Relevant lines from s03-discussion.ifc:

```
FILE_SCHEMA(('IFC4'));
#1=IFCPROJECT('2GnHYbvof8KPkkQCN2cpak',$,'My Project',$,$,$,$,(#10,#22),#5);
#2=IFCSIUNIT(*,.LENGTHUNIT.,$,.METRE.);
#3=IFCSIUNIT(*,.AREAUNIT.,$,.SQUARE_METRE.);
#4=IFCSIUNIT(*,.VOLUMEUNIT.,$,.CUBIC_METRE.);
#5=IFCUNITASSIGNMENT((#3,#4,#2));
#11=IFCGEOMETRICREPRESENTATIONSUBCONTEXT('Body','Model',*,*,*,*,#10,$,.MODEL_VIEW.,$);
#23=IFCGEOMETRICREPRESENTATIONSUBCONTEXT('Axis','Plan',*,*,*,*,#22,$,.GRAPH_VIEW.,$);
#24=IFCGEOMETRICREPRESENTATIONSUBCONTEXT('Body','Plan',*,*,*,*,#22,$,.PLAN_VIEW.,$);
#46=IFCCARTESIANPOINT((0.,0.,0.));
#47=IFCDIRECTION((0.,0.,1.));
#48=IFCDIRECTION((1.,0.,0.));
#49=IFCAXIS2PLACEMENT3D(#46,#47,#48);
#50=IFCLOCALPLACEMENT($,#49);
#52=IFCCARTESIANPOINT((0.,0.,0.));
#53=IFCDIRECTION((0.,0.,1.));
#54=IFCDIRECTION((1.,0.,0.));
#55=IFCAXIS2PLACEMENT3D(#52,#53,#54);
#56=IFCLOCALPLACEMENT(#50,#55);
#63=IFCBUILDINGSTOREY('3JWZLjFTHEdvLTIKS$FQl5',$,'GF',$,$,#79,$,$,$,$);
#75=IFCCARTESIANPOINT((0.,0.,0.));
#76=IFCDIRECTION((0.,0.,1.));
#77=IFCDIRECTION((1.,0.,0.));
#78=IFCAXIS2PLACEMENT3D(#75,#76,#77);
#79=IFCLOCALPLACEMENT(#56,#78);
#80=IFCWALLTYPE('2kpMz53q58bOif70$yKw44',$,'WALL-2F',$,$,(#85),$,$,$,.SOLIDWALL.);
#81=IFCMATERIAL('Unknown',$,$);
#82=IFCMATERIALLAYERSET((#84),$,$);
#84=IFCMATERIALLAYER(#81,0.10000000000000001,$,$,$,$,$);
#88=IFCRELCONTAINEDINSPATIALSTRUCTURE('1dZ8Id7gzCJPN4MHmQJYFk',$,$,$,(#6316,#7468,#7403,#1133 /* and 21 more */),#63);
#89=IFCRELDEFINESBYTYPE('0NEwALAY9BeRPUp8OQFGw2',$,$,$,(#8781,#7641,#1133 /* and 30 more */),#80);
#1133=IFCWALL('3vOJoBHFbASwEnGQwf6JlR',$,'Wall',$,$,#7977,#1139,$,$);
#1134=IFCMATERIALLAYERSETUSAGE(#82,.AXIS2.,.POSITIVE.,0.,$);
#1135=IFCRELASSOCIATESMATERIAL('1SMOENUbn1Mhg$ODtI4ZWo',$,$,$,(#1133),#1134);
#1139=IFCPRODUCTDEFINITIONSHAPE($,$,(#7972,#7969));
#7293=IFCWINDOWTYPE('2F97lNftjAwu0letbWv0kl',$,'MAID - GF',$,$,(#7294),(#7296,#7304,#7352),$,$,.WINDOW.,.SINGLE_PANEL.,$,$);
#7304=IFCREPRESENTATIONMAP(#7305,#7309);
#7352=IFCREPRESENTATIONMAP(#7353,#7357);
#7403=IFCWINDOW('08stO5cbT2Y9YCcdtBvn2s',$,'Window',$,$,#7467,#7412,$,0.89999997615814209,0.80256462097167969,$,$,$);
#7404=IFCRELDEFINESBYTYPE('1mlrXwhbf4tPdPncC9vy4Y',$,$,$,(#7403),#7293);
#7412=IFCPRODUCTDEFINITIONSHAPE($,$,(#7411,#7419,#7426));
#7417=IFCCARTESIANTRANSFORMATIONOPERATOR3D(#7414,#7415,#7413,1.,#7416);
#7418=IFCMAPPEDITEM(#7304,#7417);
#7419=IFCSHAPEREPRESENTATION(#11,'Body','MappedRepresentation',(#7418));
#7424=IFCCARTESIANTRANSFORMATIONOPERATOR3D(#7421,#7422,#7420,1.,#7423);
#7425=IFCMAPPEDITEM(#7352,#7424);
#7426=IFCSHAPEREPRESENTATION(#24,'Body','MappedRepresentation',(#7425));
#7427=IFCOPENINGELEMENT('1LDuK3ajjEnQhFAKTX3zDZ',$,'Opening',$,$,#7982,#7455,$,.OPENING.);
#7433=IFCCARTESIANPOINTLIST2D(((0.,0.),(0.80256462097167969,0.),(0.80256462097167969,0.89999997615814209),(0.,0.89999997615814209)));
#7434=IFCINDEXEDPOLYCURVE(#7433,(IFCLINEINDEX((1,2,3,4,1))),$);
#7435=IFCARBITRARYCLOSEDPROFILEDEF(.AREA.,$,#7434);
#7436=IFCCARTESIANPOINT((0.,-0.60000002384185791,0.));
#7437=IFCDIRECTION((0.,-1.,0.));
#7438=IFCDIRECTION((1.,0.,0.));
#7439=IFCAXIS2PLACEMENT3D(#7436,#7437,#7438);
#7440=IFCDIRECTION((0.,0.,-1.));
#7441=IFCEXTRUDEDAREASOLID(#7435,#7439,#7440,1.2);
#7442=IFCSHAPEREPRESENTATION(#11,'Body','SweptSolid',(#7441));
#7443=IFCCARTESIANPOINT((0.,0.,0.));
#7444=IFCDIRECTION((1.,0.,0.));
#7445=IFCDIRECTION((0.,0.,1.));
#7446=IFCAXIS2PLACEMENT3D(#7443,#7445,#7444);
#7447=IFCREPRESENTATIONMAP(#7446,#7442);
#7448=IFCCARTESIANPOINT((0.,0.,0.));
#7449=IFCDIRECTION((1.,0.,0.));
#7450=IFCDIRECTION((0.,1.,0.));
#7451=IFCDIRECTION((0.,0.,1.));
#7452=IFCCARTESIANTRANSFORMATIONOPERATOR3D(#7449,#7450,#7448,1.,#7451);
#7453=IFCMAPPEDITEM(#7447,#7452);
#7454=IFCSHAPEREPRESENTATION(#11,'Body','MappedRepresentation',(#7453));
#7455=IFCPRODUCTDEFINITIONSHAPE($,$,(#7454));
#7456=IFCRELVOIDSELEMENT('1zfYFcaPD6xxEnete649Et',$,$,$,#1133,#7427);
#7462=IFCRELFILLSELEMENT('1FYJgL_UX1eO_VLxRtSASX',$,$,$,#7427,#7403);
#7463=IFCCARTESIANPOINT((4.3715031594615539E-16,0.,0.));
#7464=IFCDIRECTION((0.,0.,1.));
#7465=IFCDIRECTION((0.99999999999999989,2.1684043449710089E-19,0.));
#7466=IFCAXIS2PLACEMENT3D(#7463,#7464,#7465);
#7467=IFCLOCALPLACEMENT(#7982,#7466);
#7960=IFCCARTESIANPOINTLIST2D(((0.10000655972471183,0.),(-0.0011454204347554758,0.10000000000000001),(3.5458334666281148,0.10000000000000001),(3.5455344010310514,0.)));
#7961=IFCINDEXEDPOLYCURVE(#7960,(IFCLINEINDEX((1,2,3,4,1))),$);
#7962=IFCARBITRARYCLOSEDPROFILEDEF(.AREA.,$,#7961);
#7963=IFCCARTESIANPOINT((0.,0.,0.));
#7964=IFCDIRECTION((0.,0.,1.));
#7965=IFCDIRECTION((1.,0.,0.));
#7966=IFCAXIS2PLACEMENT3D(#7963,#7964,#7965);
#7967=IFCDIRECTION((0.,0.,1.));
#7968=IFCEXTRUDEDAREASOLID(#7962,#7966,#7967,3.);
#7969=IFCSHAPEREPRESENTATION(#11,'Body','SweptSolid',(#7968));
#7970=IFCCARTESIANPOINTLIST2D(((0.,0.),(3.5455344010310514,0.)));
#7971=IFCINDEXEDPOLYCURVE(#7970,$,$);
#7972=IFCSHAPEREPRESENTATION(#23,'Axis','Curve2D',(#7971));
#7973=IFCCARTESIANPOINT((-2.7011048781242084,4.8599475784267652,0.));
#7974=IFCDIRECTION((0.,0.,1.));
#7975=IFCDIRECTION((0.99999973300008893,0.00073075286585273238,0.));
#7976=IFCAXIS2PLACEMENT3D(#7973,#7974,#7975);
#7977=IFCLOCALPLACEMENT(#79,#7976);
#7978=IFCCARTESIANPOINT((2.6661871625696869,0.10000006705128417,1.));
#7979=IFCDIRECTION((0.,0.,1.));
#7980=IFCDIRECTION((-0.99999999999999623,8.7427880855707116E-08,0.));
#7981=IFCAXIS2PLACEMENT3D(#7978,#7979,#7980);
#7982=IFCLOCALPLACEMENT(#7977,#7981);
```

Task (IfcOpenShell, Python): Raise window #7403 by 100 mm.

```python
import numpy as np
import ifcopenshell
import ifcopenshell.api.geometry
import ifcopenshell.util.placement
import ifcopenshell.util.unit

model = ifcopenshell.open("s03-discussion.ifc")
unit_scale = ifcopenshell.util.unit.calculate_unit_scale(model)

window = model.by_id(7403)
opening = window.FillsVoids[0].RelatingOpeningElement
dz = 0.1 / unit_scale

shift = np.array([0.0, 0.0, dz])
# The window is placed relative to its opening, so it follows when the opening moves.
matrix = ifcopenshell.util.placement.get_local_placement(opening.ObjectPlacement)
matrix[:3, 3] += shift
ifcopenshell.api.geometry.edit_object_placement(
    model, product=opening, matrix=matrix, is_si=False, should_transform_children=True
)

print(f"moved by {dz * unit_scale:+.3f} m")

model.write("s03-discussion_v2.ifc")
```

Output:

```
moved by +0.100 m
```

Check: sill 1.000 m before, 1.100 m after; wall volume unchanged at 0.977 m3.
